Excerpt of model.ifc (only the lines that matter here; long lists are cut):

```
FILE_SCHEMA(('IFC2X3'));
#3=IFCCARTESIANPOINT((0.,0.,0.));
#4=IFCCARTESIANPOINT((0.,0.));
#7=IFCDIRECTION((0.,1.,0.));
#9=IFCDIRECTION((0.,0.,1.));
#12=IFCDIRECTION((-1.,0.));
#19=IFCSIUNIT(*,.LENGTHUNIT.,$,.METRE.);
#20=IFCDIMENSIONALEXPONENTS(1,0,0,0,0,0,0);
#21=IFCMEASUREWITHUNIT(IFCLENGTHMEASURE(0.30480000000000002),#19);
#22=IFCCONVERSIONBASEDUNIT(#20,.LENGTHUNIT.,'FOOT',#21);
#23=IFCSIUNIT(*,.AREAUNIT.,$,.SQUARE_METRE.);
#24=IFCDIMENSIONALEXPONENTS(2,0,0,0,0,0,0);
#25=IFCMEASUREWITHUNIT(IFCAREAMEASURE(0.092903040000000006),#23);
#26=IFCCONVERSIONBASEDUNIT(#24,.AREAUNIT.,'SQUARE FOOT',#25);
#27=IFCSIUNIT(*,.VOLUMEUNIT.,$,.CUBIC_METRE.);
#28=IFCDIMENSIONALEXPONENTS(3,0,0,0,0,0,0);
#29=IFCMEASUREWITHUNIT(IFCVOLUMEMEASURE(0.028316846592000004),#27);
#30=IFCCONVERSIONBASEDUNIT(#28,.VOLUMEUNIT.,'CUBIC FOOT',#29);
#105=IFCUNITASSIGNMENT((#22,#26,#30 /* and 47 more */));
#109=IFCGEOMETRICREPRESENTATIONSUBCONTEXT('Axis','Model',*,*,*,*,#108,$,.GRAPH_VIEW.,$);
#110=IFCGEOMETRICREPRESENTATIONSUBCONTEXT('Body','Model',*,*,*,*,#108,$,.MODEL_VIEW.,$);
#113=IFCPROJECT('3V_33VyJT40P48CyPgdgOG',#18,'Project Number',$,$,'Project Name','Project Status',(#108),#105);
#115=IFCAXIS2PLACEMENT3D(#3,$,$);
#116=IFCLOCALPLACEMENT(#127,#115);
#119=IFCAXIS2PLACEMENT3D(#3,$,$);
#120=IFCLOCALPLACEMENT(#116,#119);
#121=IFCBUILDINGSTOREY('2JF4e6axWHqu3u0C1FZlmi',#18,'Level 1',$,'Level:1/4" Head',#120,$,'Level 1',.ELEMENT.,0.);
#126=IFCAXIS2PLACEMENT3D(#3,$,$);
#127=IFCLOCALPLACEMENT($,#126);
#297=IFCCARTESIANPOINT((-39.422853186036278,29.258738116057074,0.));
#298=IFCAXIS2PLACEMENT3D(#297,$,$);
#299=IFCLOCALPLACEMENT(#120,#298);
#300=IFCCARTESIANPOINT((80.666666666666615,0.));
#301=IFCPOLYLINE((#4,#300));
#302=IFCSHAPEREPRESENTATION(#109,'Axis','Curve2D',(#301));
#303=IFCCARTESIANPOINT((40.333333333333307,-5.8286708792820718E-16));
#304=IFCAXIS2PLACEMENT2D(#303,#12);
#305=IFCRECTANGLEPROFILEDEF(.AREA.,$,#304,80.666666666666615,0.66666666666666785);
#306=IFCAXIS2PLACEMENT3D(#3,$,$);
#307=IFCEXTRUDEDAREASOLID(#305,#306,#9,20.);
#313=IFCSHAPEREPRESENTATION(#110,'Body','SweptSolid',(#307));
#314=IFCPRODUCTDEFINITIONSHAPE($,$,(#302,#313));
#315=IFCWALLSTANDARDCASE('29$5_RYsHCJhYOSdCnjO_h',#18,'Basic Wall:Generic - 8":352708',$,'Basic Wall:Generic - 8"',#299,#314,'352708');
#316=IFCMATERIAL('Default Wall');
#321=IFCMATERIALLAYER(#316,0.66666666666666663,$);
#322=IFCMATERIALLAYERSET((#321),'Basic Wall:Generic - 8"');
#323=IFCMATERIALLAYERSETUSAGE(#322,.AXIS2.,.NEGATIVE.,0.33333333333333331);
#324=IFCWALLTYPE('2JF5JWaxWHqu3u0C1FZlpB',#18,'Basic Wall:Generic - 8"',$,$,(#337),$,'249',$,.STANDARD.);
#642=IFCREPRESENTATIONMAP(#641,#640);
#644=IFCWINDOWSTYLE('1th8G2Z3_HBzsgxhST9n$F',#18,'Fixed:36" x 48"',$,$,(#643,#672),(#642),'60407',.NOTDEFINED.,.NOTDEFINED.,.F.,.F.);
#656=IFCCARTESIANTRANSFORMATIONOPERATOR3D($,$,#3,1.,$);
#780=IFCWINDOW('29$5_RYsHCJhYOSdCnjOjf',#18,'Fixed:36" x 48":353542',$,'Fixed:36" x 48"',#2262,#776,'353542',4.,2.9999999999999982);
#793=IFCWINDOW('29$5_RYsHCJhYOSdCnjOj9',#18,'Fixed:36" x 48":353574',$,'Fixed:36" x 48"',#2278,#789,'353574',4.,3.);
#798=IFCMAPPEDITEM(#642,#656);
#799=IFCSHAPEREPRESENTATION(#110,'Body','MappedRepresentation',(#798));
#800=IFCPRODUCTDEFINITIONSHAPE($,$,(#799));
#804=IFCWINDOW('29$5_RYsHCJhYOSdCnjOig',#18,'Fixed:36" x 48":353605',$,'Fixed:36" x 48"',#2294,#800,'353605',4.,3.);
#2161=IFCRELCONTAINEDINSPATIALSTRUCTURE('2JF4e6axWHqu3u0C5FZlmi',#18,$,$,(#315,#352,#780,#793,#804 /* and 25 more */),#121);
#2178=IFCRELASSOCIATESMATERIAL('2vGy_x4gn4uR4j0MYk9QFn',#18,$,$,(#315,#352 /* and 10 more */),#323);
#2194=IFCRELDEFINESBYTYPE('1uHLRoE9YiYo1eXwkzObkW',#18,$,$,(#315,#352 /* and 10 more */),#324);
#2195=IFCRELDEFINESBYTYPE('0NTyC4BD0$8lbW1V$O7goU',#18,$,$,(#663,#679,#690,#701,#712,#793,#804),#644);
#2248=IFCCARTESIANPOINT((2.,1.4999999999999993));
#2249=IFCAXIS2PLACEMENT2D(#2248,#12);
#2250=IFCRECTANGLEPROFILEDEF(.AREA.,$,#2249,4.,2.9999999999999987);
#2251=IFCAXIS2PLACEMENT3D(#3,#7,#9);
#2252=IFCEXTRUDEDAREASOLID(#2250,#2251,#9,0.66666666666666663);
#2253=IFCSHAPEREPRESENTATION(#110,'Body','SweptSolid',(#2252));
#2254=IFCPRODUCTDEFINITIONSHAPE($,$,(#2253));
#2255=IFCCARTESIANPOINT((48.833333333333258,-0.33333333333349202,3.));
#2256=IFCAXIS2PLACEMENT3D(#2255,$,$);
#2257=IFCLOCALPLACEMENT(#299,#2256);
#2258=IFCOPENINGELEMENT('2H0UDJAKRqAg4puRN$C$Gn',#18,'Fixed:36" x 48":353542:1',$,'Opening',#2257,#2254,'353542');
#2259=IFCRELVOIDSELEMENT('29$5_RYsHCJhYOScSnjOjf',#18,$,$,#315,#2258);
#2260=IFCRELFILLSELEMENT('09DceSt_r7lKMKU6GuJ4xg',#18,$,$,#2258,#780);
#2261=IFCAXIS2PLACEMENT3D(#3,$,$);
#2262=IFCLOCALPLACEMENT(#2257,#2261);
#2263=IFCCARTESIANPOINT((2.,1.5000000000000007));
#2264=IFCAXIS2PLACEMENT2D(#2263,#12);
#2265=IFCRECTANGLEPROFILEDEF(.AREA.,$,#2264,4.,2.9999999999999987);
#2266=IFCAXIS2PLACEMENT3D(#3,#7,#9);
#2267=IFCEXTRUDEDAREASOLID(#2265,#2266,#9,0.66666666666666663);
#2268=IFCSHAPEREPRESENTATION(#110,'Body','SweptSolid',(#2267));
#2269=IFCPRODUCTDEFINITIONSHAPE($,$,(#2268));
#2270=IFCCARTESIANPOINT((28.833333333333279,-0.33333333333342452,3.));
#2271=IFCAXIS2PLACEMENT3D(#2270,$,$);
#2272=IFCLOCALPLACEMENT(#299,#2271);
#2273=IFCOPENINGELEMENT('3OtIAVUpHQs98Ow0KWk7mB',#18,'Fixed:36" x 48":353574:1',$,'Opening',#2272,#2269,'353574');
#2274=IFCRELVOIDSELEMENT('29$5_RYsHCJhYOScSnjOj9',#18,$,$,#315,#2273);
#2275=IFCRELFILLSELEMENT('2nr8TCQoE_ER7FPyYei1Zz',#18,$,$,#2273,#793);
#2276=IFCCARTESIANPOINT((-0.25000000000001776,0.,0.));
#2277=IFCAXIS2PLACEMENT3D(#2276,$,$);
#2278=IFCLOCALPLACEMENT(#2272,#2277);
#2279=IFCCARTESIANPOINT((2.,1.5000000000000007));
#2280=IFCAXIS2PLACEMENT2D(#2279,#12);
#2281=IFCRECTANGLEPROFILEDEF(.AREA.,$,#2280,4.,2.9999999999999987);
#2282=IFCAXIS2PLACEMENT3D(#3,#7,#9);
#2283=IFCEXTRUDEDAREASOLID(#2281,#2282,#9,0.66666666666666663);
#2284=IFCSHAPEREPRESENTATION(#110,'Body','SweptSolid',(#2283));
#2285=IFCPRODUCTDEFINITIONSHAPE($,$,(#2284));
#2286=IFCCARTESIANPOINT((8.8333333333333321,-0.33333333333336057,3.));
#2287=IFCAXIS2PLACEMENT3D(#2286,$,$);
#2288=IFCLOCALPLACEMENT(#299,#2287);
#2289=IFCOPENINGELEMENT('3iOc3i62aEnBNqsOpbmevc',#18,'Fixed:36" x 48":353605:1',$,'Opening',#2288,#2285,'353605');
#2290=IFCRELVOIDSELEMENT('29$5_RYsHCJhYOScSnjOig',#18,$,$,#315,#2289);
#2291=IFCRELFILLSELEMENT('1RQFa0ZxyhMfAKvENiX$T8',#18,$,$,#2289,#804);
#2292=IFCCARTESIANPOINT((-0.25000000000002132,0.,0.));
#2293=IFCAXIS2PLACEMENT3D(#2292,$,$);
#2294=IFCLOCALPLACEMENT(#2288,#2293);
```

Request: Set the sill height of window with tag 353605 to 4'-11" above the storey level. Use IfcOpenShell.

```python
import numpy as np
import ifcopenshell
import ifcopenshell.api.geometry
import ifcopenshell.geom
import ifcopenshell.util.element
import ifcopenshell.util.placement
import ifcopenshell.util.shape
import ifcopenshell.util.unit

model = ifcopenshell.open("model.ifc")
unit_scale = ifcopenshell.util.unit.calculate_unit_scale(model)

window = model.by_guid("29$5_RYsHCJhYOSdCnjOig")
opening = window.FillsVoids[0].RelatingOpeningElement
storey = ifcopenshell.util.element.get_container(window, ifc_class="IfcBuildingStorey")
level = ifcopenshell.util.placement.get_local_placement(storey.ObjectPlacement)[2, 3]

# The opening's origin need not be at the sill, so measure its lowest point.
shape = ifcopenshell.geom.create_shape(ifcopenshell.geom.settings(), opening)
bottom = ifcopenshell.util.shape.get_shape_bottom_elevation(shape, shape.geometry) / unit_scale
dz = level + 59 * 0.0254 / unit_scale - bottom

shift = np.array([0.0, 0.0, dz])
# The window is placed relative to its opening, so it follows when the opening moves.
matrix = ifcopenshell.util.placement.get_local_placement(opening.ObjectPlacement)
matrix[:3, 3] += shift
ifcopenshell.api.geometry.edit_object_placement(
    model, product=opening, matrix=matrix, is_si=False, should_transform_children=True
)

print(f"moved by {dz * unit_scale:+.3f} m")

model.write("model-out.ifc")
```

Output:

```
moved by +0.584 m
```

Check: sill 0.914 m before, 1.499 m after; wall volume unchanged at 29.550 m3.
